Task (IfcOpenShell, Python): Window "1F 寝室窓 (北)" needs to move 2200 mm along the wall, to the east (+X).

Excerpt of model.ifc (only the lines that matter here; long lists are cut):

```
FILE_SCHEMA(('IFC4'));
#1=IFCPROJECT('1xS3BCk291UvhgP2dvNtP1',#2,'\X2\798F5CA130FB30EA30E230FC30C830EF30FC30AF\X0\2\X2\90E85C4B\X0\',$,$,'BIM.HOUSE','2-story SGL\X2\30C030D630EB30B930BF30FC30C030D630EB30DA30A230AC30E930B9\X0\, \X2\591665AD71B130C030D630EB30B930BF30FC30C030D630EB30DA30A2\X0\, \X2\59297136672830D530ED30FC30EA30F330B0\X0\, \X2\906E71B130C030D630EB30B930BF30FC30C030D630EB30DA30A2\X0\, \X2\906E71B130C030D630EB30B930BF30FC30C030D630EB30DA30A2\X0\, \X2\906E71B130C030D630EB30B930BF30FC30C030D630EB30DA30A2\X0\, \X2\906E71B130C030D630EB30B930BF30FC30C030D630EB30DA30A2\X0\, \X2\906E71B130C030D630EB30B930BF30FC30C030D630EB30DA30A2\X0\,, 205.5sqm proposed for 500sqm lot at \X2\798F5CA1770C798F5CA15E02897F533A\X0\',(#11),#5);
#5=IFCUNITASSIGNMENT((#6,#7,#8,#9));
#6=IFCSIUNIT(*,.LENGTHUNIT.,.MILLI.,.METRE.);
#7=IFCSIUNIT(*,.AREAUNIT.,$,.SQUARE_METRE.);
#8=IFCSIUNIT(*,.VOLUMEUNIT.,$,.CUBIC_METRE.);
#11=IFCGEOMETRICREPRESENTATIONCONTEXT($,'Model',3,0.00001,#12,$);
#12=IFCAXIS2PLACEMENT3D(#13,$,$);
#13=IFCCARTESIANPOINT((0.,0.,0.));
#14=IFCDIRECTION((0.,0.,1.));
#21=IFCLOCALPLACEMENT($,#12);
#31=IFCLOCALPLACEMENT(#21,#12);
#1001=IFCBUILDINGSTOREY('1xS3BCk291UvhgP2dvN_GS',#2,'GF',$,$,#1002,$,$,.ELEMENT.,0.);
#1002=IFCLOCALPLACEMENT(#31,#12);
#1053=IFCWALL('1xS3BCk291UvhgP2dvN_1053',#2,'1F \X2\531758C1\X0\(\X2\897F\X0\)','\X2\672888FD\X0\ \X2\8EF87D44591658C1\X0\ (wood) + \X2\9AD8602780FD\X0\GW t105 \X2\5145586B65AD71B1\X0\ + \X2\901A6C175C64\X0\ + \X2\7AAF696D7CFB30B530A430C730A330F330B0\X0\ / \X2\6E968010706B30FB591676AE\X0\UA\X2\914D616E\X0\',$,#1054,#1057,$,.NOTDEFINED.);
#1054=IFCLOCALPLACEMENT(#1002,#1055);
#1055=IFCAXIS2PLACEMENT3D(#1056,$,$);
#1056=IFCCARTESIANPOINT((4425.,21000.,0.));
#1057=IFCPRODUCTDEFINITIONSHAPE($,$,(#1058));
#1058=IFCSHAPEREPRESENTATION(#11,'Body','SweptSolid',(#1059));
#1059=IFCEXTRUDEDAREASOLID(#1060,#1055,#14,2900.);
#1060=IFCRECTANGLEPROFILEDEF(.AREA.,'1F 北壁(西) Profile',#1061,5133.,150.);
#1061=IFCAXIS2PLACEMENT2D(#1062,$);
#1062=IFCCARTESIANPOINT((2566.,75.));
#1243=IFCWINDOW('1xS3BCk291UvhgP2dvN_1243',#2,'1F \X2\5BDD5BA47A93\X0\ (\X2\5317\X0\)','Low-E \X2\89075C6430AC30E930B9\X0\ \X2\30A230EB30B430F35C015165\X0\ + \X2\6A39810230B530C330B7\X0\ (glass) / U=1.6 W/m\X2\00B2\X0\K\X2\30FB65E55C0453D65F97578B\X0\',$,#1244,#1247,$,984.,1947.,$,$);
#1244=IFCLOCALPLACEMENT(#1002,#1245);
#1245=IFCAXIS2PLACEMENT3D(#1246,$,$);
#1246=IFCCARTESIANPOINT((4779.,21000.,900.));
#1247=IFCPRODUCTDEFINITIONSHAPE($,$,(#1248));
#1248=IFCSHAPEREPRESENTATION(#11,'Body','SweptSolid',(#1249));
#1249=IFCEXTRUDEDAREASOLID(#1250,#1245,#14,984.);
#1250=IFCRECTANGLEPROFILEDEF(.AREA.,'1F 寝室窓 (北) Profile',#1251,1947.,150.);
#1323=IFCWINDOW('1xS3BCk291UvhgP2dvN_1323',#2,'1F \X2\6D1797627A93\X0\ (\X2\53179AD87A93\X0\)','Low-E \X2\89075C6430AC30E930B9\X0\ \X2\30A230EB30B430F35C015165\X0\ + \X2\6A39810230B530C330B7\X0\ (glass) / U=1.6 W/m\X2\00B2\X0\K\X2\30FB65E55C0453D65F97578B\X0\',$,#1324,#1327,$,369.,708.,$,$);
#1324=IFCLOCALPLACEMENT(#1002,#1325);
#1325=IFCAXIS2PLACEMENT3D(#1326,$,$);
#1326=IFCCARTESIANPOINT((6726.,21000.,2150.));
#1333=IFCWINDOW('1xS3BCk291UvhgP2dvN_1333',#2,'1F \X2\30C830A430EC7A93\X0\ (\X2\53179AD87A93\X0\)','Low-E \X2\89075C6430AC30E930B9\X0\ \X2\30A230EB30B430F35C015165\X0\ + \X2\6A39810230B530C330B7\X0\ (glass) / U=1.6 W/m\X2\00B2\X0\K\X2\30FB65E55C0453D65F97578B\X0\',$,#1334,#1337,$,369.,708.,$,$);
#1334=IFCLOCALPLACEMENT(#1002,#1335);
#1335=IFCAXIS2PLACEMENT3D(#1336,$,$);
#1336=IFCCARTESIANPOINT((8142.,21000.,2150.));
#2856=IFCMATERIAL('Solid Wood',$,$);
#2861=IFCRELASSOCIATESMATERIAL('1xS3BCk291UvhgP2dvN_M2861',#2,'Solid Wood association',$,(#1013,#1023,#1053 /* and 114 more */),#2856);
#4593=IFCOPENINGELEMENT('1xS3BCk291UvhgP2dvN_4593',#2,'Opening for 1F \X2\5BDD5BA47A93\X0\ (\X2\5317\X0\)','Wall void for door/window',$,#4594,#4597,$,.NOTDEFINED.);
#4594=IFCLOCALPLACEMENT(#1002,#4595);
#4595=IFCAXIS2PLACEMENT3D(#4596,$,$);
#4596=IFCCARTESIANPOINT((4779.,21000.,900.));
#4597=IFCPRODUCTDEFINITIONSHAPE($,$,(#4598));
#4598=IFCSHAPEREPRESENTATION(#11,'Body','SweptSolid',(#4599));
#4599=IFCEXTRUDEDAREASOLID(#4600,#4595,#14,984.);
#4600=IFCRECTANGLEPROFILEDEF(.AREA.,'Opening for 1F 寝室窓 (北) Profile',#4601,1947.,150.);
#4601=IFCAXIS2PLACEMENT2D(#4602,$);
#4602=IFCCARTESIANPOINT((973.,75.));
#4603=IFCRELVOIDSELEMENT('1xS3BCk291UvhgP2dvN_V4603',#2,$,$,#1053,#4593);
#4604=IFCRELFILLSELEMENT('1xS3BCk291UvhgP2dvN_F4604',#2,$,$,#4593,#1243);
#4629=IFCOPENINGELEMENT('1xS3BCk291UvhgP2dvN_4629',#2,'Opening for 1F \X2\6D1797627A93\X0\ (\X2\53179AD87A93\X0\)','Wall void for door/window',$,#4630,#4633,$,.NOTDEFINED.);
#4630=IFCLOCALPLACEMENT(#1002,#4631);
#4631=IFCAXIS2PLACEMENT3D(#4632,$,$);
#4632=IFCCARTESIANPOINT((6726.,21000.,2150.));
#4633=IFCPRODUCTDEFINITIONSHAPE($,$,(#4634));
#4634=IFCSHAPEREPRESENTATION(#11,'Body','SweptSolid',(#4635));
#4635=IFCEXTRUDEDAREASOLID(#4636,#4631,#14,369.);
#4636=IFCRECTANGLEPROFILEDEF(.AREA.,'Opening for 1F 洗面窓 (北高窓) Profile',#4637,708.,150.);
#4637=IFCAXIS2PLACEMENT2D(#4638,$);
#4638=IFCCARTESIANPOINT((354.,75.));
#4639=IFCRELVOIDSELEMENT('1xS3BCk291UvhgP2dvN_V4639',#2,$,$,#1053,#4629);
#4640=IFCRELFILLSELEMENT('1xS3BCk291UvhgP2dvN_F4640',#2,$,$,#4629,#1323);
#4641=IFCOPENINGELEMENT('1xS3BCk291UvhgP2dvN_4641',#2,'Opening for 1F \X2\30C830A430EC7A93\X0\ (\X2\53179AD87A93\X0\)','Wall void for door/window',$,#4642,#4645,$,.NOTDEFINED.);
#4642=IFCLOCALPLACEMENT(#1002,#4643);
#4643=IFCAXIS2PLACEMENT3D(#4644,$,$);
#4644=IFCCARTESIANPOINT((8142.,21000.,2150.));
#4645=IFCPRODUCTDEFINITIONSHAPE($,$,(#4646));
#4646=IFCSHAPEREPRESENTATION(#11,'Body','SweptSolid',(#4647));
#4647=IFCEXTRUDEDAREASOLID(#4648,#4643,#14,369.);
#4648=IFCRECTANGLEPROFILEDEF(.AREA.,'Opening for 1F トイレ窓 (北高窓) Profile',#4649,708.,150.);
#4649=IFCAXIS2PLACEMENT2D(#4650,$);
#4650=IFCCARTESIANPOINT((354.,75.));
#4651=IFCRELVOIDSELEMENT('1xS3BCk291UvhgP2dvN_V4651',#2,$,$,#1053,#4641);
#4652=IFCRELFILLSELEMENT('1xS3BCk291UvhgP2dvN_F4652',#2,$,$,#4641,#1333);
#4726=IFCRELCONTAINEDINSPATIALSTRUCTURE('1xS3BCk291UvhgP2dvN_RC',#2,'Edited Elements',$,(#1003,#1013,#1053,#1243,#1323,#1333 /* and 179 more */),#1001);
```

```python
import ifcopenshell
import ifcopenshell.api.geometry
import ifcopenshell.util.placement
import ifcopenshell.util.unit

model = ifcopenshell.open("model.ifc")
unit_scale = ifcopenshell.util.unit.calculate_unit_scale(model)

window = model.by_guid("1xS3BCk291UvhgP2dvN_1243")
opening = window.FillsVoids[0].RelatingOpeningElement
wall = opening.VoidsElements[0].RelatingBuildingElement

wall_matrix = ifcopenshell.util.placement.get_local_placement(wall.ObjectPlacement)
shift = wall_matrix[:3, 0] * 2.2 / unit_scale
before = ifcopenshell.util.placement.get_local_placement(window.ObjectPlacement)[:3, 3].copy()

# The window is not placed relative to its opening, so move both.
for product in (opening, window):
    matrix = ifcopenshell.util.placement.get_local_placement(product.ObjectPlacement)
    matrix[:3, 3] += shift
    ifcopenshell.api.geometry.edit_object_placement(model, product=product, matrix=matrix, is_si=False)

after = ifcopenshell.util.placement.get_local_placement(window.ObjectPlacement)[:3, 3]
print("window moved by", (after - before).round(3) + 0.0)

model.write("model_rev.ifc")
```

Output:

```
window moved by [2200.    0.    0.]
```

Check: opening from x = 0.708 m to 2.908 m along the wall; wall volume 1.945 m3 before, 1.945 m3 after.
